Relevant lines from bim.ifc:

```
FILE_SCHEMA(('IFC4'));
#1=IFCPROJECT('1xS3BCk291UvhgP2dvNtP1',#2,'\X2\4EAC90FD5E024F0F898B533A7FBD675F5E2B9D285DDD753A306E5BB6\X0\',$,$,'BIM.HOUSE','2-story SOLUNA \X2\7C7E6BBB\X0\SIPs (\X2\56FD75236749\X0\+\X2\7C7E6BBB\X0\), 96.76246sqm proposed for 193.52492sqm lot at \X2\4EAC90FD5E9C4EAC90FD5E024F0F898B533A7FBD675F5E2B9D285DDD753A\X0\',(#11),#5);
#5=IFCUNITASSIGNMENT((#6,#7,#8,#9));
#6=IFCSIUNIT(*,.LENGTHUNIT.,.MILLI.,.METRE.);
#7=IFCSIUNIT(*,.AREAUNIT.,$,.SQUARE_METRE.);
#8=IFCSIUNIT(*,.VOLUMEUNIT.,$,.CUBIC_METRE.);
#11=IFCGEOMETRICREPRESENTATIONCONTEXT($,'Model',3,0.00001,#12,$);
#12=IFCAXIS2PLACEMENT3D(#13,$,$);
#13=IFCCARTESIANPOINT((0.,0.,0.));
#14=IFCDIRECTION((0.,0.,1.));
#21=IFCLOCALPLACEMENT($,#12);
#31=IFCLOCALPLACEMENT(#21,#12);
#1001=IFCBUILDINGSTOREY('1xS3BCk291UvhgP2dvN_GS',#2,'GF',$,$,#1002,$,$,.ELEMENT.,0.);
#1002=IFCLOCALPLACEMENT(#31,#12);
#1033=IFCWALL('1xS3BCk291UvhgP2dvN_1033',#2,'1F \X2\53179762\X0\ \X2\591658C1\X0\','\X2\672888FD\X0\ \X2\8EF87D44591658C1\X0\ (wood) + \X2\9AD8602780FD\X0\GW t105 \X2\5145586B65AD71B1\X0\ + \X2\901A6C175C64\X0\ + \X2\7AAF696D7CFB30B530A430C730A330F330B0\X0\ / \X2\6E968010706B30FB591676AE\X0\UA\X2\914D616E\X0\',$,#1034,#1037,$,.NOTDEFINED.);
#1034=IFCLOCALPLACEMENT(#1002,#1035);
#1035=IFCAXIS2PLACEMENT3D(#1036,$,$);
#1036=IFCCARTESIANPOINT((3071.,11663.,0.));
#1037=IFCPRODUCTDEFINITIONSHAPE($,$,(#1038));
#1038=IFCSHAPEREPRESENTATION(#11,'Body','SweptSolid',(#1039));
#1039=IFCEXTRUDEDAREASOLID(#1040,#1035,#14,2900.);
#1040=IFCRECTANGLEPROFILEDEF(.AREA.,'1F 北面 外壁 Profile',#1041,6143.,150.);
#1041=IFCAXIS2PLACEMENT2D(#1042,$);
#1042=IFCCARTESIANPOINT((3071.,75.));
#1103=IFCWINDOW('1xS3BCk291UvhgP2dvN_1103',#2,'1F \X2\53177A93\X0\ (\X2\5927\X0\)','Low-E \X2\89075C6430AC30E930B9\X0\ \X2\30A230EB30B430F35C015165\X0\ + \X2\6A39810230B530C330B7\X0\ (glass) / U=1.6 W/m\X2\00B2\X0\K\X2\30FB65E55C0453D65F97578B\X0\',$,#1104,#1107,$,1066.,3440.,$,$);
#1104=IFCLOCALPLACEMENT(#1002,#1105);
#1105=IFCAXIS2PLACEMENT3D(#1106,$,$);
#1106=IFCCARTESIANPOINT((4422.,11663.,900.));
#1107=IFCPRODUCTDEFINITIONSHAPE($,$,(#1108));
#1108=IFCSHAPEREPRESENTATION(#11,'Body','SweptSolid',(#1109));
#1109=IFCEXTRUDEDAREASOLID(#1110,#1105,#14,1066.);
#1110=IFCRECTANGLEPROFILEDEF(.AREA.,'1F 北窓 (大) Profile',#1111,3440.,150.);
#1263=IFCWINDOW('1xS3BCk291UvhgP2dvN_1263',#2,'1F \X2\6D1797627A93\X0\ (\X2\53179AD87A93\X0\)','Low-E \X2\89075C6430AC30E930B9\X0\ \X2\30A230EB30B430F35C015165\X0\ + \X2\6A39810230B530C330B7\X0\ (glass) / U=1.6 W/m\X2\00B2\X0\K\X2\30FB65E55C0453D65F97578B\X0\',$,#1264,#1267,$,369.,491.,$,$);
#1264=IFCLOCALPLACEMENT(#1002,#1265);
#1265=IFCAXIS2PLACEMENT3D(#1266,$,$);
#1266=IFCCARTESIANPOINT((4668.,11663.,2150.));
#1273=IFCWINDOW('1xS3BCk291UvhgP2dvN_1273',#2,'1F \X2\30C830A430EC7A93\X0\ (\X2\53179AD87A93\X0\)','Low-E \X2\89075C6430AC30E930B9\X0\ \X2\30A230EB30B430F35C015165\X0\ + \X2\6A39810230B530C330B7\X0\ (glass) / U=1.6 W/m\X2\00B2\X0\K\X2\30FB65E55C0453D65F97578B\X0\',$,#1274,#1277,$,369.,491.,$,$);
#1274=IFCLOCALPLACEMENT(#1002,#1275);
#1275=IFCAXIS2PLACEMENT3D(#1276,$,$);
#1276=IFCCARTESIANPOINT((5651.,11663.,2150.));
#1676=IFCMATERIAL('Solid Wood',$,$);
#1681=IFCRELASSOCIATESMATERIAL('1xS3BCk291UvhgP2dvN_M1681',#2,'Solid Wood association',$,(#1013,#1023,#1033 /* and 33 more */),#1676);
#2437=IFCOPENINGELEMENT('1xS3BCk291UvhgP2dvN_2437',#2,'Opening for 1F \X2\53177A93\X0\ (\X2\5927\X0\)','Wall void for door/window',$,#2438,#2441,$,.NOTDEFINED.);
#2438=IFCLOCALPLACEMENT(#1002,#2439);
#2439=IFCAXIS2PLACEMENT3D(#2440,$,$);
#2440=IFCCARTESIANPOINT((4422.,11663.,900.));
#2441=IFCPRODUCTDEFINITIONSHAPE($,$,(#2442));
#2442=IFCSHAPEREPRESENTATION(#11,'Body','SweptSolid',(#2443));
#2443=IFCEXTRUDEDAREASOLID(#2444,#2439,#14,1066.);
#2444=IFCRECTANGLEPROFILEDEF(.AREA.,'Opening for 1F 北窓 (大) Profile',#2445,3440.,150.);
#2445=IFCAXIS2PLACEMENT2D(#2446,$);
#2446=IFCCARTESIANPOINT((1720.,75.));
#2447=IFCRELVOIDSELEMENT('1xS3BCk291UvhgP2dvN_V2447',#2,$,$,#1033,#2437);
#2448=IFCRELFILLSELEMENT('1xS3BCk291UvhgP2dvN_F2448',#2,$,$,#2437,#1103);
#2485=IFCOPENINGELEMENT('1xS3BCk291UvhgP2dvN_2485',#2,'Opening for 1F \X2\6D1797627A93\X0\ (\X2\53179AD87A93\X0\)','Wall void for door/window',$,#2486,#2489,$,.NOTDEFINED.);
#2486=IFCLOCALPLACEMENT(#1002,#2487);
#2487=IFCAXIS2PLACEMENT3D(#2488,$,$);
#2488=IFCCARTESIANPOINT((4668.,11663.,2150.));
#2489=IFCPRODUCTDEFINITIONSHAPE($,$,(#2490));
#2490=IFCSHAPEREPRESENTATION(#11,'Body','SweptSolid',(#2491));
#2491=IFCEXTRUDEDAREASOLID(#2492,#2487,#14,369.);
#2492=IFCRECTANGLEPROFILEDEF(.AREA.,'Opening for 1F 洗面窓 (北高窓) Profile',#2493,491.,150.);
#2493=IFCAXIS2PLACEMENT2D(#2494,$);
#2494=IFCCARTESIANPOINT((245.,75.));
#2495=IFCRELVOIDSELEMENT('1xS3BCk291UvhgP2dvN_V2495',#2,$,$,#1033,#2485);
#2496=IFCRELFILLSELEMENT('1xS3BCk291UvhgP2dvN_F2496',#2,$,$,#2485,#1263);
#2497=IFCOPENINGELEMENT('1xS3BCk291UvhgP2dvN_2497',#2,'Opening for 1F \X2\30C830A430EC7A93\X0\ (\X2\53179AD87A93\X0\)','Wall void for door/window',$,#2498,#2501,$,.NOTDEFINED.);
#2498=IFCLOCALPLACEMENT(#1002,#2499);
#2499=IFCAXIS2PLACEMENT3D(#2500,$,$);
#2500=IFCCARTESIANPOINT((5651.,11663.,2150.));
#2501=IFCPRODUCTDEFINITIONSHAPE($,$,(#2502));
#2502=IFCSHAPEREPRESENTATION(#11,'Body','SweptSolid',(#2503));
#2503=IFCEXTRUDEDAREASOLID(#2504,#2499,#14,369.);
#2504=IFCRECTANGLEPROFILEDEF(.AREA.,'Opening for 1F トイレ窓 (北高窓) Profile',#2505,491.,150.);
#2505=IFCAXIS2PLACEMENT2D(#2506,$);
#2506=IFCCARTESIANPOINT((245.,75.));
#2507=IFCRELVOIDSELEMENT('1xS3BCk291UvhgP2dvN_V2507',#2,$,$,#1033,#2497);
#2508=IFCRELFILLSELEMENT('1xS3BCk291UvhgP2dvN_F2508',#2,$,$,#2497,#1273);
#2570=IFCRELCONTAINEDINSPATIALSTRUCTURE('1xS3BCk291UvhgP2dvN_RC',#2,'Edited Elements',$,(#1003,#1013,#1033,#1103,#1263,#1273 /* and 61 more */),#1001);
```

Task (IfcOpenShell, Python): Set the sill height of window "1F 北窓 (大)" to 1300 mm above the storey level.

```python
import numpy as np
import ifcopenshell
import ifcopenshell.api.geometry
import ifcopenshell.geom
import ifcopenshell.util.element
import ifcopenshell.util.placement
import ifcopenshell.util.shape
import ifcopenshell.util.unit

model = ifcopenshell.open("bim.ifc")
unit_scale = ifcopenshell.util.unit.calculate_unit_scale(model)

window = model.by_guid("1xS3BCk291UvhgP2dvN_1103")
opening = window.FillsVoids[0].RelatingOpeningElement
storey = ifcopenshell.util.element.get_container(window, ifc_class="IfcBuildingStorey")
level = ifcopenshell.util.placement.get_local_placement(storey.ObjectPlacement)[2, 3]

# The opening's origin need not be at the sill, so measure its lowest point.
shape = ifcopenshell.geom.create_shape(ifcopenshell.geom.settings(), opening)
bottom = ifcopenshell.util.shape.get_shape_bottom_elevation(shape, shape.geometry) / unit_scale
dz = level + 1300.0 - bottom

shift = np.array([0.0, 0.0, dz])
# The window is not placed relative to its opening, so move both.
for product in (opening, window):
    matrix = ifcopenshell.util.placement.get_local_placement(product.ObjectPlacement)
    matrix[:3, 3] += shift
    ifcopenshell.api.geometry.edit_object_placement(model, product=product, matrix=matrix, is_si=False)

print(f"moved by {dz * unit_scale:+.3f} m")

model.write("bim_v2.ifc")
```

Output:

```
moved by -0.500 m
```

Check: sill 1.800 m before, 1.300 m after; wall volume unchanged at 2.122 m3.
